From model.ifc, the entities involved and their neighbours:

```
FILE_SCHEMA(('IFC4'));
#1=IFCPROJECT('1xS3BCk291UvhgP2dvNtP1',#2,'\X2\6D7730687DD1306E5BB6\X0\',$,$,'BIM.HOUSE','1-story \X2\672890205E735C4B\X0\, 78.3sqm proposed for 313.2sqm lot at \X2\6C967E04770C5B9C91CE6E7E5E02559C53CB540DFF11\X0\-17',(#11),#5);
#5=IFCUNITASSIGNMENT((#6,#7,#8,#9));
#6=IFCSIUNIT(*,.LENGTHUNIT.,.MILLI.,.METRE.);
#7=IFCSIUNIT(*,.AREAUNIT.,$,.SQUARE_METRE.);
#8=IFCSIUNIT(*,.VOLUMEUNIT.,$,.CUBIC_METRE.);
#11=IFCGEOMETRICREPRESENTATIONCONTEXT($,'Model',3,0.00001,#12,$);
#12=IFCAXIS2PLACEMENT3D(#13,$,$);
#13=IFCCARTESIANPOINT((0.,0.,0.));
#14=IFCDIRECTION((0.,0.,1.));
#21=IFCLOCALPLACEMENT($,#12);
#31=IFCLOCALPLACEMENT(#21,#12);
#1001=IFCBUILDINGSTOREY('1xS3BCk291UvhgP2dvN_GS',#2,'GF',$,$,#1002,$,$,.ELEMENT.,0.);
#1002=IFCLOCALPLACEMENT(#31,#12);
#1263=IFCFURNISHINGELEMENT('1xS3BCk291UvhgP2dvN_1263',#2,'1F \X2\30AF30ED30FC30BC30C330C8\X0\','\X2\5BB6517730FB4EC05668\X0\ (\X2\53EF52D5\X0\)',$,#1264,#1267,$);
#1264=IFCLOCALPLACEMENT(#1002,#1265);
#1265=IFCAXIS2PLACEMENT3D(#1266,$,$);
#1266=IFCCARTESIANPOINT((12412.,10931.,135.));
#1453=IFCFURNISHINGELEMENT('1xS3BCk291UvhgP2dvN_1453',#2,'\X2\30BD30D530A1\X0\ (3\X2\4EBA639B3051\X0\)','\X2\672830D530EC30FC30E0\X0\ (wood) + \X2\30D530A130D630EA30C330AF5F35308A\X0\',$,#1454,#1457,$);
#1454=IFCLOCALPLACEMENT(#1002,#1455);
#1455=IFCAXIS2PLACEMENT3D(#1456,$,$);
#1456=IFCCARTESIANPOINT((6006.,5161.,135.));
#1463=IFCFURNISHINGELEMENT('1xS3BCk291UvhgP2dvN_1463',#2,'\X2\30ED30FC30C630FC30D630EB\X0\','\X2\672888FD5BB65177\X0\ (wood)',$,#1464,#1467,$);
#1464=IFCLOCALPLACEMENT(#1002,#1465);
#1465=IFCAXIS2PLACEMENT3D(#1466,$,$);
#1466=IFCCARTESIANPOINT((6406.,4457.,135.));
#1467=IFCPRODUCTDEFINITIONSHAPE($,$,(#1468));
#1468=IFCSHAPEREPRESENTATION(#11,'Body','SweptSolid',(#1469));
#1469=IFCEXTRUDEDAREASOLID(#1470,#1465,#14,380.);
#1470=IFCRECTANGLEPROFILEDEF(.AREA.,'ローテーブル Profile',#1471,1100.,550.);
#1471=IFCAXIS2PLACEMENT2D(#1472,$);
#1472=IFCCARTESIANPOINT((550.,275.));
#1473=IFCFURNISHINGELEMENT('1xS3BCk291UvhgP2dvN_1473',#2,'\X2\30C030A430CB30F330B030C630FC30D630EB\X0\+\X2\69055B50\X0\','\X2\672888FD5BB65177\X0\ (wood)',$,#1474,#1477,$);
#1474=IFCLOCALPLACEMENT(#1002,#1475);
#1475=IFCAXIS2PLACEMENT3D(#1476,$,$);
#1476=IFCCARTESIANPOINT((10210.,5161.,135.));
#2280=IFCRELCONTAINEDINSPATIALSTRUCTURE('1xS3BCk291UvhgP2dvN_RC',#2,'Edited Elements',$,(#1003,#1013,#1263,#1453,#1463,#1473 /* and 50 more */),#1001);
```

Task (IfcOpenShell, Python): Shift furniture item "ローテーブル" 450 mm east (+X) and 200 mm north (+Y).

```python
import ifcopenshell
import ifcopenshell.api.geometry
import ifcopenshell.util.placement
import ifcopenshell.util.unit

model = ifcopenshell.open("model.ifc")
unit_scale = ifcopenshell.util.unit.calculate_unit_scale(model)

item = model.by_guid("1xS3BCk291UvhgP2dvN_1463")
matrix = ifcopenshell.util.placement.get_local_placement(item.ObjectPlacement)
matrix[0, 3] += 0.45 / unit_scale
matrix[1, 3] += 0.2 / unit_scale
ifcopenshell.api.geometry.edit_object_placement(model, product=item, matrix=matrix, is_si=False)

print(ifcopenshell.util.placement.get_local_placement(item.ObjectPlacement).round(3) + 0.0)

model.write("model_v2.ifc")
```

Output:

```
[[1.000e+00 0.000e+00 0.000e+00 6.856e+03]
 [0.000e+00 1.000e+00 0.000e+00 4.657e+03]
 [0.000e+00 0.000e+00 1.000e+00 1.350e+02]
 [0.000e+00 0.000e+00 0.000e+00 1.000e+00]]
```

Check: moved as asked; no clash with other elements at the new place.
